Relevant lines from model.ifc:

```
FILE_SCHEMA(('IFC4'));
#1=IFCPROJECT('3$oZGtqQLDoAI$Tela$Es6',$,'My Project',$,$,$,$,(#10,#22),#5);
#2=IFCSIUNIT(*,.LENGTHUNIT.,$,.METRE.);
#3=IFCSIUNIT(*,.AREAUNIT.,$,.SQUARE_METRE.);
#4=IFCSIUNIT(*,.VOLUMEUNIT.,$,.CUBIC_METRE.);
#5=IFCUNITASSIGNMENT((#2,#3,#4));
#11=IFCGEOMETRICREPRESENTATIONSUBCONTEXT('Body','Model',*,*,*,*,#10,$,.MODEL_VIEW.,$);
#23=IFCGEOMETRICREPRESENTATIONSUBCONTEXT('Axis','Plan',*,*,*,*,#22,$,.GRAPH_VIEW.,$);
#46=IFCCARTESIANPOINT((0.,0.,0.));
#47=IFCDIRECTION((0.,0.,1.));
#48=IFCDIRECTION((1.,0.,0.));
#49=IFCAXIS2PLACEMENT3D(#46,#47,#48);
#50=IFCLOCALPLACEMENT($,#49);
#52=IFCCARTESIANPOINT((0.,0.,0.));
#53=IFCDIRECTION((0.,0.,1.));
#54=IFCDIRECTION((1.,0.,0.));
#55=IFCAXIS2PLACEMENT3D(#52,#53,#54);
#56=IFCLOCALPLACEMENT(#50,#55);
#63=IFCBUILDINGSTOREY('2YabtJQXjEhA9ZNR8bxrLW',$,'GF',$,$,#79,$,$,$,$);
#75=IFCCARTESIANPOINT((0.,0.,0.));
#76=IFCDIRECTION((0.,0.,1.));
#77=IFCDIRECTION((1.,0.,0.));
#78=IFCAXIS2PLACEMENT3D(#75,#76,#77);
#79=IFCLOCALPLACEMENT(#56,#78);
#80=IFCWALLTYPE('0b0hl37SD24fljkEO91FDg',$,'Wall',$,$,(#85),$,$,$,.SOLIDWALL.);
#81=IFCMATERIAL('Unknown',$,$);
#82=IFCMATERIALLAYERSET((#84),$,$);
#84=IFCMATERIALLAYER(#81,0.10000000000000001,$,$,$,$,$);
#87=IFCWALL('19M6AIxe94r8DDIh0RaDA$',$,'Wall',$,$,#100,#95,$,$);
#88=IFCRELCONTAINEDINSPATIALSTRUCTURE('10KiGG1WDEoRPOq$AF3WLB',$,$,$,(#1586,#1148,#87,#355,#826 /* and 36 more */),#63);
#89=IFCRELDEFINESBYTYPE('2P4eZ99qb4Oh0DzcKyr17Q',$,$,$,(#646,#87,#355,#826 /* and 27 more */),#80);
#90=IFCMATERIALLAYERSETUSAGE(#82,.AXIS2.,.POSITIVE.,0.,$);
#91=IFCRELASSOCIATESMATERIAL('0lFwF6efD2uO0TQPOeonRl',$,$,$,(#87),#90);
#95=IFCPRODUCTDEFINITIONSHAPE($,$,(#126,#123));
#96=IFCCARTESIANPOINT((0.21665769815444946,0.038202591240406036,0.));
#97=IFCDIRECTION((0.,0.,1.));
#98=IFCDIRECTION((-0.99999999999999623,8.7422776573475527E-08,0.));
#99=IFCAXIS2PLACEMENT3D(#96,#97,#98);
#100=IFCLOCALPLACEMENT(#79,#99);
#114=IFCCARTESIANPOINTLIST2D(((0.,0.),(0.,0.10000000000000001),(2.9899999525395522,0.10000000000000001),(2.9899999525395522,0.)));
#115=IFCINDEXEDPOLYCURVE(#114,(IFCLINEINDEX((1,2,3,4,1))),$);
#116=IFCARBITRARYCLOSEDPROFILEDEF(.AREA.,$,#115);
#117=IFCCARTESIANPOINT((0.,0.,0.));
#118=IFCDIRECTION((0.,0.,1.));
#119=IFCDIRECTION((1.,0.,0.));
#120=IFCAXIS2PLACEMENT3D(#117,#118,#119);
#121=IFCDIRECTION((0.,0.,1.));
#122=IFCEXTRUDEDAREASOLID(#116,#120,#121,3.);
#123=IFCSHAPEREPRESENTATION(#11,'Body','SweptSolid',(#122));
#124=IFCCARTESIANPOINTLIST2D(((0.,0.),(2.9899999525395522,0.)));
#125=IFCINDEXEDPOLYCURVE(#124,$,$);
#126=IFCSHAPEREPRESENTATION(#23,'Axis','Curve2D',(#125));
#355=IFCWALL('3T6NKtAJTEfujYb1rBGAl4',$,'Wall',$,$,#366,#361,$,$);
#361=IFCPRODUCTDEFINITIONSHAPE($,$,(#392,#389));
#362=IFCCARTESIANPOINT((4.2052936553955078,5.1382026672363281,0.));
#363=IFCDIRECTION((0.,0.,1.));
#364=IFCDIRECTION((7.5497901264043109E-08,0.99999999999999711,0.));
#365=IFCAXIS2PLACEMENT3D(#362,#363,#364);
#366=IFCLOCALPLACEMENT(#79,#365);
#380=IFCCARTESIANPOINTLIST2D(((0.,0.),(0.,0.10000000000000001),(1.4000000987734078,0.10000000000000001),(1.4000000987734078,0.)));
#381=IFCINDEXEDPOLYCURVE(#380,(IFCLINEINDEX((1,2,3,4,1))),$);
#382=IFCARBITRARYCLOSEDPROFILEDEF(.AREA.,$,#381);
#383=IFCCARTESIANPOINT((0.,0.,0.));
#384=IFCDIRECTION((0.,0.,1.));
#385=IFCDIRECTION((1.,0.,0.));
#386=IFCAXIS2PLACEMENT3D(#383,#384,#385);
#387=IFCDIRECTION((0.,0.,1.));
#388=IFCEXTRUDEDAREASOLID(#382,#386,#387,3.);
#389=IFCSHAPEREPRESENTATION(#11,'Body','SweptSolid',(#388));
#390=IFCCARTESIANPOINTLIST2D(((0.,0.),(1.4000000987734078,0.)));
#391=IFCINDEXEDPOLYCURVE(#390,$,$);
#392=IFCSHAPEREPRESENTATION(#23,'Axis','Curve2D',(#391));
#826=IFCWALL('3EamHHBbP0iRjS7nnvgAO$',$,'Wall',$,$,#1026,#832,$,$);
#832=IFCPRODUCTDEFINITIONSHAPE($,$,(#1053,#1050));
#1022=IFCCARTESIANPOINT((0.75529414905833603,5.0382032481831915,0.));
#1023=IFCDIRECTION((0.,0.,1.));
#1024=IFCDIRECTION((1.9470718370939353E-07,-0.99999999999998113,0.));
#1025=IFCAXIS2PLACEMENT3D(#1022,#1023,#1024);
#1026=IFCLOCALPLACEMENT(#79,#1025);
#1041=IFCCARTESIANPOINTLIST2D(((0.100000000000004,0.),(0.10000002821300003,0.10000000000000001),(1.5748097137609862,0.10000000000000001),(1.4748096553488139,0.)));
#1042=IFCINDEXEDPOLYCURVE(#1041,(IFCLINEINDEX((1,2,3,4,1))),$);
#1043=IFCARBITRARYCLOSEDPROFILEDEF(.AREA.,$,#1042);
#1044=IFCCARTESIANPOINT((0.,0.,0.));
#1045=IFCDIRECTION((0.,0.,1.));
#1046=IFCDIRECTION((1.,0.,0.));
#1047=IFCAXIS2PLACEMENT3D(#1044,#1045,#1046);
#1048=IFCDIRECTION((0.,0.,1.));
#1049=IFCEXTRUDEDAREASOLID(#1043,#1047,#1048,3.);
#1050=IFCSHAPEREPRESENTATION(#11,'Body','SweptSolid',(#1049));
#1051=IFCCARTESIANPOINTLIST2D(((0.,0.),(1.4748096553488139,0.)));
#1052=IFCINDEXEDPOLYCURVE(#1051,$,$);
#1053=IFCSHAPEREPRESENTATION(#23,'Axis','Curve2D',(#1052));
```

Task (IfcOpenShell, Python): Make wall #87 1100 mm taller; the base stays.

```python
import ifcopenshell
import ifcopenshell.geom
import ifcopenshell.util.representation
import ifcopenshell.util.shape
import ifcopenshell.util.unit

model = ifcopenshell.open("model.ifc")
unit_scale = ifcopenshell.util.unit.calculate_unit_scale(model)
settings = ifcopenshell.geom.settings()


def volume(element):
    """Net volume in cubic metres, openings subtracted."""
    shape = ifcopenshell.geom.create_shape(settings, element)
    return ifcopenshell.util.shape.get_volume(shape.geometry)


wall = model.by_guid("19M6AIxe94r8DDIh0RaDA$")
before = volume(wall)

body = ifcopenshell.util.representation.get_representation(wall, "Model", "Body")
solid = body.Items[0]
old_height = solid.Depth
solid.Depth += 1.1 / unit_scale
after = volume(wall)

print(f"height {old_height:g} -> {solid.Depth:g}, volume {before:.3f} -> {after:.3f} m3")

model.write("model_edited.ifc")
```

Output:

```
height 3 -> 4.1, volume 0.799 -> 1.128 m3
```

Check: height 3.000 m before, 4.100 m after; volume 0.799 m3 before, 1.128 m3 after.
